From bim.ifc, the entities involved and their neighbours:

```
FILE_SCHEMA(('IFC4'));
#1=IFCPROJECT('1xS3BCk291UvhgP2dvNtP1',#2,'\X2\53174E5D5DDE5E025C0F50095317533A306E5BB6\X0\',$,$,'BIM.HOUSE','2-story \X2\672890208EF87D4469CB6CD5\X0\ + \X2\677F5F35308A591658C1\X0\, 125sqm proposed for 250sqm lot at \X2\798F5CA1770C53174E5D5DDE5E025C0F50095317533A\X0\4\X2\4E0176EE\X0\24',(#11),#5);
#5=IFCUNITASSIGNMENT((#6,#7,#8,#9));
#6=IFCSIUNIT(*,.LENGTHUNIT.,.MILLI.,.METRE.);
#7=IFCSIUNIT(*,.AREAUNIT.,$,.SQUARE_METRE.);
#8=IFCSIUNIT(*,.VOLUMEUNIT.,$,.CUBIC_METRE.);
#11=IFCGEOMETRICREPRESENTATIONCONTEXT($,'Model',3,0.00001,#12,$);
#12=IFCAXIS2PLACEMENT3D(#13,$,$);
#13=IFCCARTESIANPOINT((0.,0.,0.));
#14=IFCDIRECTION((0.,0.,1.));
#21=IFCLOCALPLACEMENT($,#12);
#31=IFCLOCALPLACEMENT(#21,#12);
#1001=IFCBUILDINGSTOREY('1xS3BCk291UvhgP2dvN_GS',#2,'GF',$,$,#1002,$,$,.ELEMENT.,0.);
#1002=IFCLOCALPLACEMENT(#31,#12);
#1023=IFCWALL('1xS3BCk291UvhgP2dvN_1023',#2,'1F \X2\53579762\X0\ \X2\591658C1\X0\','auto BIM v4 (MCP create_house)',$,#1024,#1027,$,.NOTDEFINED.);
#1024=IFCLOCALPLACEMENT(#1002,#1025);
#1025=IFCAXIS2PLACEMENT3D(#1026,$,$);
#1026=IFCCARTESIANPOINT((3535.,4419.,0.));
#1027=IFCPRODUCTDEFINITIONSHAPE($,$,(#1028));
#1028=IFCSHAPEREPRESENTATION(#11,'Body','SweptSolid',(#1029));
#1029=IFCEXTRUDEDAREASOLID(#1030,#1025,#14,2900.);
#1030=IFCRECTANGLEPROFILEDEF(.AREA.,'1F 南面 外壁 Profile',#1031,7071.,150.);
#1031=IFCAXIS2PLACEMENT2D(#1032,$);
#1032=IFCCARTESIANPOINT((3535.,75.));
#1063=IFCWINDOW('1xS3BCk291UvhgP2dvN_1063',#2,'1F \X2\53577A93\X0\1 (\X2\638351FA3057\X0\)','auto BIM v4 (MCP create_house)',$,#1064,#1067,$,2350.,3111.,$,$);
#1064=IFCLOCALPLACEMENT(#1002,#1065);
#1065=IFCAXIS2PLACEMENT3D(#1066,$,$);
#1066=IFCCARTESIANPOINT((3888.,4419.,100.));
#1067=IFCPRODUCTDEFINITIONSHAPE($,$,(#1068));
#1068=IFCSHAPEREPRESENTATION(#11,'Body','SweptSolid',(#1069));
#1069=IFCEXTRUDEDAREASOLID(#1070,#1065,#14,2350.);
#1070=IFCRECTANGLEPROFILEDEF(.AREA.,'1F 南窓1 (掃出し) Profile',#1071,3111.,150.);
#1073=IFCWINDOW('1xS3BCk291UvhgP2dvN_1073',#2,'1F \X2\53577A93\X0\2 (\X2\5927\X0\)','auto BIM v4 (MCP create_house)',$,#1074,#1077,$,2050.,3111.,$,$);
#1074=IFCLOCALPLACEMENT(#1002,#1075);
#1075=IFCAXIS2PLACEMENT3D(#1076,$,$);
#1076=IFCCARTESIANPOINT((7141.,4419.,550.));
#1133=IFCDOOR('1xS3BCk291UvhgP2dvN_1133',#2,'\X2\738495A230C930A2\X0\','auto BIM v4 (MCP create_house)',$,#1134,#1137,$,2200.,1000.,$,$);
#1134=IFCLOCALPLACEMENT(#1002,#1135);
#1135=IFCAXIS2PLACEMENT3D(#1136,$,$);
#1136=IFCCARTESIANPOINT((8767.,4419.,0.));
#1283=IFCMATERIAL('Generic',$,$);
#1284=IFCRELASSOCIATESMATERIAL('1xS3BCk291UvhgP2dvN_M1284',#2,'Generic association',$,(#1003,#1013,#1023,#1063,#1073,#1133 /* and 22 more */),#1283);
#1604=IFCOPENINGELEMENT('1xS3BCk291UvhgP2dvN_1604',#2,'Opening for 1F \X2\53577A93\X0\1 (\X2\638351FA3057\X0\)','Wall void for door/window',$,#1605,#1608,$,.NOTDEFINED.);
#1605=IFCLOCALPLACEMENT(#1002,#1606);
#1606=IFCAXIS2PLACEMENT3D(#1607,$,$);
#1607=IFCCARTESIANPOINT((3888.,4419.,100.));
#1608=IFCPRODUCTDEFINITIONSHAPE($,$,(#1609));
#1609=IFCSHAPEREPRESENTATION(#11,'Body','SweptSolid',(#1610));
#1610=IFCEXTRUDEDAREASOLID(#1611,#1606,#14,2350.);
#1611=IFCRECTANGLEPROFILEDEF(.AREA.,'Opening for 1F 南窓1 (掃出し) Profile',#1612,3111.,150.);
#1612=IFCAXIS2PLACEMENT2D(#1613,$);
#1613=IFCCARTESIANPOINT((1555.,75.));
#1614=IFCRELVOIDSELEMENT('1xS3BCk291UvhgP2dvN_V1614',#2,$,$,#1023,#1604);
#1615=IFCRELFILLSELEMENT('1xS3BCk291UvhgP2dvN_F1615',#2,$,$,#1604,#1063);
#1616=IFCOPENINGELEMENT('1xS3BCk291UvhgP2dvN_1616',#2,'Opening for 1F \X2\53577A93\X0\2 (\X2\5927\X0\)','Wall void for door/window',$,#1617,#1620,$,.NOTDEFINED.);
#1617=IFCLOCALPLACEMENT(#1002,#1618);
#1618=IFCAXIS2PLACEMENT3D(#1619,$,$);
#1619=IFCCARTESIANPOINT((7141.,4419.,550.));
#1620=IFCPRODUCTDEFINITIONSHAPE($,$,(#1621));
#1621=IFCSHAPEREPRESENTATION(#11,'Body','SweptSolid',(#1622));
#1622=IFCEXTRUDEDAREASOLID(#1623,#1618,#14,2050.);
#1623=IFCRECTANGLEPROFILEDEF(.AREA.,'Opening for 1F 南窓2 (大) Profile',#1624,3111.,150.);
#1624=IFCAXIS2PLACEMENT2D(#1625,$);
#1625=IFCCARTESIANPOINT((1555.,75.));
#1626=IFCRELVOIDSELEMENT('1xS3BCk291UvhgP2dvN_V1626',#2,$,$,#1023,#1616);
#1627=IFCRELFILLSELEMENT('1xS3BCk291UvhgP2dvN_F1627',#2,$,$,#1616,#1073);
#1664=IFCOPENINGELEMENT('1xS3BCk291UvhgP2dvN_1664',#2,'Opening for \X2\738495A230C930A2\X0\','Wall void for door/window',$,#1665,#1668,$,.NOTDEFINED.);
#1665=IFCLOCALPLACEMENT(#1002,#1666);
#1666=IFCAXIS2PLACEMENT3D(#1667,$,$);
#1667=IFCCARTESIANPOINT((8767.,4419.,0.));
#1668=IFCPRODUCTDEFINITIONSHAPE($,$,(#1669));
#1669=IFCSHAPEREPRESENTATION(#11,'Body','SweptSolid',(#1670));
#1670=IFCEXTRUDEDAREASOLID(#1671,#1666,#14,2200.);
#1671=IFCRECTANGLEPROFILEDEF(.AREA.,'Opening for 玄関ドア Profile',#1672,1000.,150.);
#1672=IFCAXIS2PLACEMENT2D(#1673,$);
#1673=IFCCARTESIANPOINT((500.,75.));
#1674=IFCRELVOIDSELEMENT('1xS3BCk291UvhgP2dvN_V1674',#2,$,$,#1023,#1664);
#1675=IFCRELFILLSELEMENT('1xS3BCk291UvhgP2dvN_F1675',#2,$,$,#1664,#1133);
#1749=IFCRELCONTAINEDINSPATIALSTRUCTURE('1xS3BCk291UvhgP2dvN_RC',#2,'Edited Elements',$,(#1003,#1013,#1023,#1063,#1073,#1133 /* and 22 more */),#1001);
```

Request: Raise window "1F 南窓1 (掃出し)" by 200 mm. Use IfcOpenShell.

```python
import numpy as np
import ifcopenshell
import ifcopenshell.api.geometry
import ifcopenshell.util.placement
import ifcopenshell.util.unit

model = ifcopenshell.open("bim.ifc")
unit_scale = ifcopenshell.util.unit.calculate_unit_scale(model)

window = model.by_id(1063)
opening = window.FillsVoids[0].RelatingOpeningElement
dz = 0.2 / unit_scale

shift = np.array([0.0, 0.0, dz])
# The window is not placed relative to its opening, so move both.
for product in (opening, window):
    matrix = ifcopenshell.util.placement.get_local_placement(product.ObjectPlacement)
    matrix[:3, 3] += shift
    ifcopenshell.api.geometry.edit_object_placement(model, product=product, matrix=matrix, is_si=False)

print(f"moved by {dz * unit_scale:+.3f} m")

model.write("bim_rev.ifc")
```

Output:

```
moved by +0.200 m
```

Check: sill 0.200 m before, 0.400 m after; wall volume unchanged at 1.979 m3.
